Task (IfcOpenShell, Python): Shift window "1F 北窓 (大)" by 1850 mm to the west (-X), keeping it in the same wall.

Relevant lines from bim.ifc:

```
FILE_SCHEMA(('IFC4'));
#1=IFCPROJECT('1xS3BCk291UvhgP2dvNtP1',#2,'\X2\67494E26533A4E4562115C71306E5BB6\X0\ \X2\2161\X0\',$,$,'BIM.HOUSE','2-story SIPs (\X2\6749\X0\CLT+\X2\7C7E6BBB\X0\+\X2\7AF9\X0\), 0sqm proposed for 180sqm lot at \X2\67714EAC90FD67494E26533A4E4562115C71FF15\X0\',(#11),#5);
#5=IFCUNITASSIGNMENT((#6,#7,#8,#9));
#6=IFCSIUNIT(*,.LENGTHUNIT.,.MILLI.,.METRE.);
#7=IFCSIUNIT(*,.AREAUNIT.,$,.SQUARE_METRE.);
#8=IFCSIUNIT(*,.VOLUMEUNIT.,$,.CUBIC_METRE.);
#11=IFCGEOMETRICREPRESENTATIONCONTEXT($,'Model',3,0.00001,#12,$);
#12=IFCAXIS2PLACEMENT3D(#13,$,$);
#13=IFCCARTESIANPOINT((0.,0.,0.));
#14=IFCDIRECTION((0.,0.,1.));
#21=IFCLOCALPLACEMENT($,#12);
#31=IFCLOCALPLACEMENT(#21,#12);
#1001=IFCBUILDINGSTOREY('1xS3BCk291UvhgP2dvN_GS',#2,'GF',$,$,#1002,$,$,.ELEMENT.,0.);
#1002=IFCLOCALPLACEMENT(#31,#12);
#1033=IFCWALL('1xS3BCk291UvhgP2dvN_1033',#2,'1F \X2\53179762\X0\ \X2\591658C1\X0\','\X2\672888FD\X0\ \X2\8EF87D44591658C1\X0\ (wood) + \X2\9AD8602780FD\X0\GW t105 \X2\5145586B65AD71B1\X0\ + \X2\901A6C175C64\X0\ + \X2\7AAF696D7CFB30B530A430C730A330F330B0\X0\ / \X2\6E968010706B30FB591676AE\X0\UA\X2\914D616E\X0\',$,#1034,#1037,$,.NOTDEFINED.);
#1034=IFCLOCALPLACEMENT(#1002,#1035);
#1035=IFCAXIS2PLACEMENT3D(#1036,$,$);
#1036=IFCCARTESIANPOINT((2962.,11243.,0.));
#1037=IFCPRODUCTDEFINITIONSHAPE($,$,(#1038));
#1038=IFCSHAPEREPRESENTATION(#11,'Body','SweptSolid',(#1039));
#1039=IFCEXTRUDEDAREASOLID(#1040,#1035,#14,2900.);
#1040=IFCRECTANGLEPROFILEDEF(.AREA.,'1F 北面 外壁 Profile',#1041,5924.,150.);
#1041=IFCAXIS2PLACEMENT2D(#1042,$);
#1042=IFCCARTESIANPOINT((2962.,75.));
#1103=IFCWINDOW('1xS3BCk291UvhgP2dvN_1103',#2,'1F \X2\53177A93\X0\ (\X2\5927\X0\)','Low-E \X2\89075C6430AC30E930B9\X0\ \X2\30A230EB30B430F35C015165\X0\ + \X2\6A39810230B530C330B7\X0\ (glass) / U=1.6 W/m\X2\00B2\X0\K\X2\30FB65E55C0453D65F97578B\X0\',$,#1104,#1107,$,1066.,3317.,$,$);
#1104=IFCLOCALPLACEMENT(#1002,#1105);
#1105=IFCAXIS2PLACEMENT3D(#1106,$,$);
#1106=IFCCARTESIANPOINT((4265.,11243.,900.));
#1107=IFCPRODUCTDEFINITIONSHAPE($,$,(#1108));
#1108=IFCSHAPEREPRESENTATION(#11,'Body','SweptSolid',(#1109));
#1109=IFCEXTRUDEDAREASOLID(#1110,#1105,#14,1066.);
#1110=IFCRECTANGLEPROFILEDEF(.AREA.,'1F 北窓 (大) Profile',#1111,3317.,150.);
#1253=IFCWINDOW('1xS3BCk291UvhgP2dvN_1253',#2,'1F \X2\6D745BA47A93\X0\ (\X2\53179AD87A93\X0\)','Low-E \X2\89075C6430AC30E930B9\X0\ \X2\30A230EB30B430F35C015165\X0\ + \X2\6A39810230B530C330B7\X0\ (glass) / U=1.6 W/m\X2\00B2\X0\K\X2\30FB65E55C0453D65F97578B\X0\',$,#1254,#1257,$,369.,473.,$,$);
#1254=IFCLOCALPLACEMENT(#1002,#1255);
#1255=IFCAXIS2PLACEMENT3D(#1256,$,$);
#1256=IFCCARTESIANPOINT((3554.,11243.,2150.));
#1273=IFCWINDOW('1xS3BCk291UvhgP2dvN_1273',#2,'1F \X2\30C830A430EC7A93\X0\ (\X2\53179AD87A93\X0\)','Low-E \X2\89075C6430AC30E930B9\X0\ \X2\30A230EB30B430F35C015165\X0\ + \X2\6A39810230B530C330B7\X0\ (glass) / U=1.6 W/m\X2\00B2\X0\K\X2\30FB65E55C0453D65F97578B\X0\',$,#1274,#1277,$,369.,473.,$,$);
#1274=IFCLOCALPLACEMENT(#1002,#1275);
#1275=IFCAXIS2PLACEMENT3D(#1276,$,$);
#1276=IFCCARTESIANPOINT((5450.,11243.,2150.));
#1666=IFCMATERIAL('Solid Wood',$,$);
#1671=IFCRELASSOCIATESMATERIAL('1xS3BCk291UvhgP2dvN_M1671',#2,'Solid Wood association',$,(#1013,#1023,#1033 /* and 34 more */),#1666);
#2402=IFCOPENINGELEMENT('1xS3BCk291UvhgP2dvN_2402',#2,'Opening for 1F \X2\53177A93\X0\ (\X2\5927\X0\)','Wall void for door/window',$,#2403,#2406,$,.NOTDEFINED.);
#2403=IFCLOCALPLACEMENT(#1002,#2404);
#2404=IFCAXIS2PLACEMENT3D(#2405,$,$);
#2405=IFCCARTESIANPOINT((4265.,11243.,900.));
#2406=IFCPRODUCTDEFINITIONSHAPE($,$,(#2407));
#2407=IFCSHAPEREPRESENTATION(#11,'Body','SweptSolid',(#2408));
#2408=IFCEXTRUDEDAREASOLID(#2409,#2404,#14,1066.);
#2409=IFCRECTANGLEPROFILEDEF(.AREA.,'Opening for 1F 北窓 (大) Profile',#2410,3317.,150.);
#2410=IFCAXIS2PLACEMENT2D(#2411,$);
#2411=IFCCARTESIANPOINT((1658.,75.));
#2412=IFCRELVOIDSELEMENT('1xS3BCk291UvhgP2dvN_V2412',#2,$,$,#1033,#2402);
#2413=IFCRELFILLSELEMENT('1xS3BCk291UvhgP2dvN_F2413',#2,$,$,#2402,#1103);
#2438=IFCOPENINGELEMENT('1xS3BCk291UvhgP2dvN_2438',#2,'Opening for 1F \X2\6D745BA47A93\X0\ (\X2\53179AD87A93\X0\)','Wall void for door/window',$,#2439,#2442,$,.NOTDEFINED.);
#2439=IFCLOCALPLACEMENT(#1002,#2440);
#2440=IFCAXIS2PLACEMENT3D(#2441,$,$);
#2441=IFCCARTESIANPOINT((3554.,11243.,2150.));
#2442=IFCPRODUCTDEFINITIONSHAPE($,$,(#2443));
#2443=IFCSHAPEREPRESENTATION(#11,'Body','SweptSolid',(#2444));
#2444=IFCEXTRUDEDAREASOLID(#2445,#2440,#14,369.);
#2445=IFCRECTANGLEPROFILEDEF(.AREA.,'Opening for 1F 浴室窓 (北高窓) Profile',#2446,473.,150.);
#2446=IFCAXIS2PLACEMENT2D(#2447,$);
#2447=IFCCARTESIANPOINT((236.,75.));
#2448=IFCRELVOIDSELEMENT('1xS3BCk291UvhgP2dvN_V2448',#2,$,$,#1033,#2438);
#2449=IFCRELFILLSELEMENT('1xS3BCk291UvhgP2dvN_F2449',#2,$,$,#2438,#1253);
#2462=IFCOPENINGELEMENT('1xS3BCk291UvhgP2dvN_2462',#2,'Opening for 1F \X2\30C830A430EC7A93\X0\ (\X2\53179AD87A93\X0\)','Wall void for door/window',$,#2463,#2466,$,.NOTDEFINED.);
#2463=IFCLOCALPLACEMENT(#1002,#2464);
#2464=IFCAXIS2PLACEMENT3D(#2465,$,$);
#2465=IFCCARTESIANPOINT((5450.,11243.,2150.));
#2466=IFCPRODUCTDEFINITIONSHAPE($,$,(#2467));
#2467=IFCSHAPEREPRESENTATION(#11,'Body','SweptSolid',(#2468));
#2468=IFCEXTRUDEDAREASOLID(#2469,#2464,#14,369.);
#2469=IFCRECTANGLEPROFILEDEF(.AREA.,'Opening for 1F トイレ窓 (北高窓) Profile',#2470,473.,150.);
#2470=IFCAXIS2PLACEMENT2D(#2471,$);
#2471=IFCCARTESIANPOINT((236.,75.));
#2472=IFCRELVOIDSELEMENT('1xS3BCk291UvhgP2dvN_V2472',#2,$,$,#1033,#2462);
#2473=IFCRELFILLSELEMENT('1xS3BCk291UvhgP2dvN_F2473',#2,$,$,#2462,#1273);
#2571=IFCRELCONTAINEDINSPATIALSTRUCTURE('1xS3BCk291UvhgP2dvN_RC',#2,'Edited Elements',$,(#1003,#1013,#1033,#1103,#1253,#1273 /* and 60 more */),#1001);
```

```python
import ifcopenshell
import ifcopenshell.api.geometry
import ifcopenshell.util.placement

model = ifcopenshell.open("bim.ifc")

window = model.by_guid("1xS3BCk291UvhgP2dvN_1103")
opening = window.FillsVoids[0].RelatingOpeningElement
wall = opening.VoidsElements[0].RelatingBuildingElement

wall_matrix = ifcopenshell.util.placement.get_local_placement(wall.ObjectPlacement)
shift = wall_matrix[:3, 0] * -1850.0
before = ifcopenshell.util.placement.get_local_placement(window.ObjectPlacement)[:3, 3].copy()

# The window is not placed relative to its opening, so move both.
for product in (opening, window):
    matrix = ifcopenshell.util.placement.get_local_placement(product.ObjectPlacement)
    matrix[:3, 3] += shift
    ifcopenshell.api.geometry.edit_object_placement(model, product=product, matrix=matrix, is_si=False)

after = ifcopenshell.util.placement.get_local_placement(window.ObjectPlacement)[:3, 3]
print("window moved by", (after - before).round(3) + 0.0)

model.write("bim_rev.ifc")
```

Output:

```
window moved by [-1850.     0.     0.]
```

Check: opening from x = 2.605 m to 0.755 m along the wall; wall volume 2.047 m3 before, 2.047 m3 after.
